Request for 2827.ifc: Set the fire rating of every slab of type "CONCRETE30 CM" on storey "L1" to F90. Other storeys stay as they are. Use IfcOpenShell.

First a look at what the model holds.

```python
import ifcopenshell
import ifcopenshell.util.element

model = ifcopenshell.open("2827.ifc")
print(model.schema)
storey = next(s for s in model.by_type("IfcBuildingStorey") if s.Name == "L1")
slabs = [e for e in ifcopenshell.util.element.get_decomposition(storey) if e.is_a("IfcSlab")]
seen = {}
for e in slabs:
    element_type = ifcopenshell.util.element.get_type(e)
    key = (element_type.Name if element_type != e and element_type else None, ifcopenshell.util.element.get_pset(e, "Pset_SlabCommon", "FireRating"))
    seen[key] = seen.get(key, 0) + 1
for (name, value), count in sorted(seen.items(), key=str):
    print(count, "x", name, "|", value)
```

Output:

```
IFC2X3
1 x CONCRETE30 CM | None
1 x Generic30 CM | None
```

```python
import ifcopenshell
import ifcopenshell.api.pset
import ifcopenshell.util.element

model = ifcopenshell.open("2827.ifc")

storey = next(s for s in model.by_type("IfcBuildingStorey") if s.Name == "L1")
slabs = [e for e in ifcopenshell.util.element.get_decomposition(storey) if e.is_a("IfcSlab")]

count = 0
for e in slabs:
    element_type = ifcopenshell.util.element.get_type(e)
    if element_type in (None, e) or element_type.Name != "CONCRETE30 CM":
        continue
    # add_pset returns the element's existing set when there is one.
    pset = ifcopenshell.api.pset.add_pset(model, product=e, name="Pset_SlabCommon")
    ifcopenshell.api.pset.edit_pset(model, pset=pset, properties={"FireRating": "F90"})
    count += 1

print(count, "slabs updated")

model.write("2827_edited.ifc")
```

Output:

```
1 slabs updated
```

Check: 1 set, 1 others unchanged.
